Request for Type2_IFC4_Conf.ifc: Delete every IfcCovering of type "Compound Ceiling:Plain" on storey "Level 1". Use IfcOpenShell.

First a look at what the model holds.

```python
import ifcopenshell
import ifcopenshell.util.element

model = ifcopenshell.open("Type2_IFC4_Conf.ifc")
print(model.schema)
storey = next(s for s in model.by_type("IfcBuildingStorey") if s.Name == "Level 1")
coverings = [e for e in ifcopenshell.util.element.get_decomposition(storey) if e.is_a("IfcCovering")]
seen = {}
for e in coverings:
    element_type = ifcopenshell.util.element.get_type(e)
    name = element_type.Name if element_type not in (None, e) else None
    seen[name] = seen.get(name, 0) + 1
for name, count in sorted(seen.items(), key=str):
    print(count, "x", name)
```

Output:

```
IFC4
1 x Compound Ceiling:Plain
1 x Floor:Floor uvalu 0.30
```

```python
import ifcopenshell
import ifcopenshell.api.root
import ifcopenshell.util.element

model = ifcopenshell.open("Type2_IFC4_Conf.ifc")

storey = next(s for s in model.by_type("IfcBuildingStorey") if s.Name == "Level 1")
coverings = [e for e in ifcopenshell.util.element.get_decomposition(storey) if e.is_a("IfcCovering")]
targets = [e for e in coverings if (t := ifcopenshell.util.element.get_type(e)) not in (None, e) and t.Name == "Compound Ceiling:Plain"]

for e in targets:
    ifcopenshell.api.root.remove_product(model, product=e)
print(len(targets), "removed")

model.write("Type2_IFC4_Conf-out.ifc")
```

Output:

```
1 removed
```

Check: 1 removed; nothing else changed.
